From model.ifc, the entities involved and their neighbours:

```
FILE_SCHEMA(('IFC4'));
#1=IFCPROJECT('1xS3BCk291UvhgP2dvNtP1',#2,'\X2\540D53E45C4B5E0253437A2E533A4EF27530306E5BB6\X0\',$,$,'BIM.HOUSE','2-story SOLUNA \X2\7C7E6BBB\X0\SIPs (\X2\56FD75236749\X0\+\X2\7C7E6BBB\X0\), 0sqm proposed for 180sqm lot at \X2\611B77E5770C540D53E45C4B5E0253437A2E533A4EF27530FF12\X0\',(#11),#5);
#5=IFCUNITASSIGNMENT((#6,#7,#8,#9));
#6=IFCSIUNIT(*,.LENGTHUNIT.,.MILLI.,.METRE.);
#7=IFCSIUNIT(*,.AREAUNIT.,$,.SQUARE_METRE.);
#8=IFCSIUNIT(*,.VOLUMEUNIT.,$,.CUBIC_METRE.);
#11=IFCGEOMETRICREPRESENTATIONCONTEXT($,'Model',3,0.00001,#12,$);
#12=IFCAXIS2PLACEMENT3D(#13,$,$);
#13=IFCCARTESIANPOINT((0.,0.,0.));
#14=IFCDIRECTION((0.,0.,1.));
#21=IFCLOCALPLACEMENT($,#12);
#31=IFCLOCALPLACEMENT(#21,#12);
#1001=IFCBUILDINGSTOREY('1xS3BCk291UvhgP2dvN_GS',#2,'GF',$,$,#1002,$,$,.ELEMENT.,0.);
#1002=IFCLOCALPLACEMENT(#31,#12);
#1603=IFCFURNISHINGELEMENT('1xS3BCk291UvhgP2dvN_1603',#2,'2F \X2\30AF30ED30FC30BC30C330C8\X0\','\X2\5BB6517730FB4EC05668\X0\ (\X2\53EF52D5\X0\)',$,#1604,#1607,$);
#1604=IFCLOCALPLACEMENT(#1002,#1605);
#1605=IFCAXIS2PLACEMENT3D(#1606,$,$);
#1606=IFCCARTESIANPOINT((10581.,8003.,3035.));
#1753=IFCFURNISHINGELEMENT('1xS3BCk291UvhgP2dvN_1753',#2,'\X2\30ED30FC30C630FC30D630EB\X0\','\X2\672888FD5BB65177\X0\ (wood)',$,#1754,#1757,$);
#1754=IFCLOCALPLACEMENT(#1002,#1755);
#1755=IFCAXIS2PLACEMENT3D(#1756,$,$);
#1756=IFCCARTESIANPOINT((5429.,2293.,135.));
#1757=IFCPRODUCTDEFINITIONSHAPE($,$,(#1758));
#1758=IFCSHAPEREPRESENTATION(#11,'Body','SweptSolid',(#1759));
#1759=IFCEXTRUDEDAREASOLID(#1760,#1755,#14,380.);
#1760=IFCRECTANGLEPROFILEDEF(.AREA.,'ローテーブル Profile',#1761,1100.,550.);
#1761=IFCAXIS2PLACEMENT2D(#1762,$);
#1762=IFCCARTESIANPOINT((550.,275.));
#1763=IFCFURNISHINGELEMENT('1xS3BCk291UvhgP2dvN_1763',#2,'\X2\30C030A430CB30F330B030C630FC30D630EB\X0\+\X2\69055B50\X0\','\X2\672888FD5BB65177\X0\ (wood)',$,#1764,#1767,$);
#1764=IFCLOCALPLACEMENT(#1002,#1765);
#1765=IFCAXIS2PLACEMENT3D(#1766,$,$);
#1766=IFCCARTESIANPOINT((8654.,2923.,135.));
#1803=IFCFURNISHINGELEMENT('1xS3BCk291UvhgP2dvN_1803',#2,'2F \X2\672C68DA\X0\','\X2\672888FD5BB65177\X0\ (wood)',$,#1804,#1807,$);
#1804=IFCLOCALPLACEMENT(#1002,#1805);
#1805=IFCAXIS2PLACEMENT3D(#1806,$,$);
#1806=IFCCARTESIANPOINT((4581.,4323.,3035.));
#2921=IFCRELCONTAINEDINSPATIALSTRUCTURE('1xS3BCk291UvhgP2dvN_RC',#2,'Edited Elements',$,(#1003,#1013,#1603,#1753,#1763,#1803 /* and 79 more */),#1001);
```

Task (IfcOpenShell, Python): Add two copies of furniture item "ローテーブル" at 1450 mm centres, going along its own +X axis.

```python
import ifcopenshell
import ifcopenshell.api.geometry
import ifcopenshell.api.root
import ifcopenshell.util.element
import ifcopenshell.util.placement
import ifcopenshell.util.unit

model = ifcopenshell.open("model.ifc")
unit_scale = ifcopenshell.util.unit.calculate_unit_scale(model)


def reuse_history(source, copy):
    """copy_class also copies each property set's owner history, people and application; keep the originals."""
    for rel in copy.IsDefinedBy:
        if rel.is_a("IfcRelDefinesByProperties") and (history := rel.RelatingPropertyDefinition.OwnerHistory):
            rel.RelatingPropertyDefinition.OwnerHistory = source.OwnerHistory
            ifcopenshell.util.element.remove_deep2(model, history)


source = model.by_guid("1xS3BCk291UvhgP2dvN_1753")
base = ifcopenshell.util.placement.get_local_placement(source.ObjectPlacement)
step = base[:3, 0] * 1.45 / unit_scale

for i in range(1, 3):
    copy = ifcopenshell.api.root.copy_class(model, product=source)
    copy.Representation = ifcopenshell.util.element.copy_deep(
        model, source.Representation, exclude=["IfcGeometricRepresentationContext", "IfcRepresentationMap"]
    )
    reuse_history(source, copy)
    matrix = base.copy()
    matrix[:3, 3] += i * step
    print("added at", matrix[:3, 3].round(3) + 0.0)
    ifcopenshell.api.geometry.edit_object_placement(model, product=copy, matrix=matrix, is_si=False)

model.write("model_v2.ifc")
```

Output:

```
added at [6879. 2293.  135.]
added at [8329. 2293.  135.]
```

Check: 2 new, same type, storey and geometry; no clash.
